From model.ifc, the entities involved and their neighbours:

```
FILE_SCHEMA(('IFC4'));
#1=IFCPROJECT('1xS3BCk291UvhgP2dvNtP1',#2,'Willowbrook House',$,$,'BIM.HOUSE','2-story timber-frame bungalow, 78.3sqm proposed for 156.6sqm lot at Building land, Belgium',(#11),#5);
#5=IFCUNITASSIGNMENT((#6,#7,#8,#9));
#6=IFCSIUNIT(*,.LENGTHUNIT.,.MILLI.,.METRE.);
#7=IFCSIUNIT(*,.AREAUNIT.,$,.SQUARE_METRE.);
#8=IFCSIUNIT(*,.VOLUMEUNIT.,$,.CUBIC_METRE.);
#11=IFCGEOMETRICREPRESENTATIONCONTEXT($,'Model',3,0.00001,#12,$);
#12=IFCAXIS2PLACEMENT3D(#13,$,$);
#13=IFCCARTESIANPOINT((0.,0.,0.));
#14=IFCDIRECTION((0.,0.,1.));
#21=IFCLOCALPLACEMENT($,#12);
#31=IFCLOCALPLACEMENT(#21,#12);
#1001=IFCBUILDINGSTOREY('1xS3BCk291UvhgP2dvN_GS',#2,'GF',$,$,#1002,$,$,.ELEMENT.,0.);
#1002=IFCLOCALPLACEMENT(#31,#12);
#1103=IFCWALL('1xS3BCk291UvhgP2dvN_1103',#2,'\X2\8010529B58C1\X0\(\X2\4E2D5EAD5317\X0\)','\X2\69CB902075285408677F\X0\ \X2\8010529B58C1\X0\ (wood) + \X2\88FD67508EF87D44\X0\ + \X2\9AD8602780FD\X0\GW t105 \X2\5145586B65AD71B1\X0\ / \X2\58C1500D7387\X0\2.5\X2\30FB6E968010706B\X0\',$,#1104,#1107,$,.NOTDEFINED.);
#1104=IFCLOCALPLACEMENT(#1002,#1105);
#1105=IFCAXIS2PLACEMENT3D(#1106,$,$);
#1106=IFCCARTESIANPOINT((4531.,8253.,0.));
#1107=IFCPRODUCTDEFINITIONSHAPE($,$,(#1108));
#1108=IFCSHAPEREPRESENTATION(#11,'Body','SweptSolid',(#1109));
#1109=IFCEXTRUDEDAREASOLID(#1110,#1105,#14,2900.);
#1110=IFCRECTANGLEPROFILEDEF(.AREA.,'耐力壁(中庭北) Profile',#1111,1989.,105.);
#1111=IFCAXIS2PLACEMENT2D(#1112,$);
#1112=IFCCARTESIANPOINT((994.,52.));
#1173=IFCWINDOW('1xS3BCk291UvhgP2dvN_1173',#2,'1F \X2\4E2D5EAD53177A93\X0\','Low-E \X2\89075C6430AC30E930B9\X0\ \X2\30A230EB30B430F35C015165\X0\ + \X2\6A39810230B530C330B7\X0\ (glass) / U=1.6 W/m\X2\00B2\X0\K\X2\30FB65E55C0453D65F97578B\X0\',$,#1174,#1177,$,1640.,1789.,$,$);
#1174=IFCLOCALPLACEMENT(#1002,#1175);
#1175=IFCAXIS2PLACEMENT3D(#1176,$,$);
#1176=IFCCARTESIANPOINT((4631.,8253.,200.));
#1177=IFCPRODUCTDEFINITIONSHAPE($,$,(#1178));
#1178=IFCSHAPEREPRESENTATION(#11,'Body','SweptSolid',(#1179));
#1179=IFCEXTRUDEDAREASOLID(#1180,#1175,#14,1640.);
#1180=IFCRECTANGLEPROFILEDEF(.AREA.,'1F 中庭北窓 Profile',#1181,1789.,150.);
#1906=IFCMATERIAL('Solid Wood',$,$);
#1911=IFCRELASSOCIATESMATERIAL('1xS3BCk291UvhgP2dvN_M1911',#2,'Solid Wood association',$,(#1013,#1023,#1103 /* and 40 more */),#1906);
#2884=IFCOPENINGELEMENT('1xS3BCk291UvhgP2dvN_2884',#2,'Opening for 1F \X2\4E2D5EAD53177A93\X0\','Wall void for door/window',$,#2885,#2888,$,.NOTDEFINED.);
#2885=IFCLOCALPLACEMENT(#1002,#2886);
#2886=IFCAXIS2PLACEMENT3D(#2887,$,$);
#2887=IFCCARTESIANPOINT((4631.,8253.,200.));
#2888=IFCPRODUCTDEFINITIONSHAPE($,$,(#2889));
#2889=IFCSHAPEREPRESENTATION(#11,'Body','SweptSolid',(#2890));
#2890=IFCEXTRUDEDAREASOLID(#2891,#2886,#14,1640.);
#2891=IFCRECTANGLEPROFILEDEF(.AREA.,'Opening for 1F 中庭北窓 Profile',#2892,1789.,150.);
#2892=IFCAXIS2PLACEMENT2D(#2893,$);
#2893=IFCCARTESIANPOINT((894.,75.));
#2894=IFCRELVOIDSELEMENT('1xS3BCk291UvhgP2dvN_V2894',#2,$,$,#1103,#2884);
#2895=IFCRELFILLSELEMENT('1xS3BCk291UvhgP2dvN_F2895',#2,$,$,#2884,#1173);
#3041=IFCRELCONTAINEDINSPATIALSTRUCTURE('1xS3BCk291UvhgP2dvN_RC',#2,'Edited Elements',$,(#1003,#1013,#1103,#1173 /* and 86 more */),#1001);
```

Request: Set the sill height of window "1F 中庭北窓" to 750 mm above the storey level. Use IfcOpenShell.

```python
import numpy as np
import ifcopenshell
import ifcopenshell.api.geometry
import ifcopenshell.geom
import ifcopenshell.util.element
import ifcopenshell.util.placement
import ifcopenshell.util.shape
import ifcopenshell.util.unit

model = ifcopenshell.open("model.ifc")
unit_scale = ifcopenshell.util.unit.calculate_unit_scale(model)

window = model.by_guid("1xS3BCk291UvhgP2dvN_1173")
opening = window.FillsVoids[0].RelatingOpeningElement
storey = ifcopenshell.util.element.get_container(window, ifc_class="IfcBuildingStorey")
level = ifcopenshell.util.placement.get_local_placement(storey.ObjectPlacement)[2, 3]

# The opening's origin need not be at the sill, so measure its lowest point.
shape = ifcopenshell.geom.create_shape(ifcopenshell.geom.settings(), opening)
bottom = ifcopenshell.util.shape.get_shape_bottom_elevation(shape, shape.geometry) / unit_scale
dz = level + 0.75 / unit_scale - bottom

shift = np.array([0.0, 0.0, dz])
# The window is not placed relative to its opening, so move both.
for product in (opening, window):
    matrix = ifcopenshell.util.placement.get_local_placement(product.ObjectPlacement)
    matrix[:3, 3] += shift
    ifcopenshell.api.geometry.edit_object_placement(model, product=product, matrix=matrix, is_si=False)

print(f"moved by {dz * unit_scale:+.3f} m")

model.write("model-out.ifc")
```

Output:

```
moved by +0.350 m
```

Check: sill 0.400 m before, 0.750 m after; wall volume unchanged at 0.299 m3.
